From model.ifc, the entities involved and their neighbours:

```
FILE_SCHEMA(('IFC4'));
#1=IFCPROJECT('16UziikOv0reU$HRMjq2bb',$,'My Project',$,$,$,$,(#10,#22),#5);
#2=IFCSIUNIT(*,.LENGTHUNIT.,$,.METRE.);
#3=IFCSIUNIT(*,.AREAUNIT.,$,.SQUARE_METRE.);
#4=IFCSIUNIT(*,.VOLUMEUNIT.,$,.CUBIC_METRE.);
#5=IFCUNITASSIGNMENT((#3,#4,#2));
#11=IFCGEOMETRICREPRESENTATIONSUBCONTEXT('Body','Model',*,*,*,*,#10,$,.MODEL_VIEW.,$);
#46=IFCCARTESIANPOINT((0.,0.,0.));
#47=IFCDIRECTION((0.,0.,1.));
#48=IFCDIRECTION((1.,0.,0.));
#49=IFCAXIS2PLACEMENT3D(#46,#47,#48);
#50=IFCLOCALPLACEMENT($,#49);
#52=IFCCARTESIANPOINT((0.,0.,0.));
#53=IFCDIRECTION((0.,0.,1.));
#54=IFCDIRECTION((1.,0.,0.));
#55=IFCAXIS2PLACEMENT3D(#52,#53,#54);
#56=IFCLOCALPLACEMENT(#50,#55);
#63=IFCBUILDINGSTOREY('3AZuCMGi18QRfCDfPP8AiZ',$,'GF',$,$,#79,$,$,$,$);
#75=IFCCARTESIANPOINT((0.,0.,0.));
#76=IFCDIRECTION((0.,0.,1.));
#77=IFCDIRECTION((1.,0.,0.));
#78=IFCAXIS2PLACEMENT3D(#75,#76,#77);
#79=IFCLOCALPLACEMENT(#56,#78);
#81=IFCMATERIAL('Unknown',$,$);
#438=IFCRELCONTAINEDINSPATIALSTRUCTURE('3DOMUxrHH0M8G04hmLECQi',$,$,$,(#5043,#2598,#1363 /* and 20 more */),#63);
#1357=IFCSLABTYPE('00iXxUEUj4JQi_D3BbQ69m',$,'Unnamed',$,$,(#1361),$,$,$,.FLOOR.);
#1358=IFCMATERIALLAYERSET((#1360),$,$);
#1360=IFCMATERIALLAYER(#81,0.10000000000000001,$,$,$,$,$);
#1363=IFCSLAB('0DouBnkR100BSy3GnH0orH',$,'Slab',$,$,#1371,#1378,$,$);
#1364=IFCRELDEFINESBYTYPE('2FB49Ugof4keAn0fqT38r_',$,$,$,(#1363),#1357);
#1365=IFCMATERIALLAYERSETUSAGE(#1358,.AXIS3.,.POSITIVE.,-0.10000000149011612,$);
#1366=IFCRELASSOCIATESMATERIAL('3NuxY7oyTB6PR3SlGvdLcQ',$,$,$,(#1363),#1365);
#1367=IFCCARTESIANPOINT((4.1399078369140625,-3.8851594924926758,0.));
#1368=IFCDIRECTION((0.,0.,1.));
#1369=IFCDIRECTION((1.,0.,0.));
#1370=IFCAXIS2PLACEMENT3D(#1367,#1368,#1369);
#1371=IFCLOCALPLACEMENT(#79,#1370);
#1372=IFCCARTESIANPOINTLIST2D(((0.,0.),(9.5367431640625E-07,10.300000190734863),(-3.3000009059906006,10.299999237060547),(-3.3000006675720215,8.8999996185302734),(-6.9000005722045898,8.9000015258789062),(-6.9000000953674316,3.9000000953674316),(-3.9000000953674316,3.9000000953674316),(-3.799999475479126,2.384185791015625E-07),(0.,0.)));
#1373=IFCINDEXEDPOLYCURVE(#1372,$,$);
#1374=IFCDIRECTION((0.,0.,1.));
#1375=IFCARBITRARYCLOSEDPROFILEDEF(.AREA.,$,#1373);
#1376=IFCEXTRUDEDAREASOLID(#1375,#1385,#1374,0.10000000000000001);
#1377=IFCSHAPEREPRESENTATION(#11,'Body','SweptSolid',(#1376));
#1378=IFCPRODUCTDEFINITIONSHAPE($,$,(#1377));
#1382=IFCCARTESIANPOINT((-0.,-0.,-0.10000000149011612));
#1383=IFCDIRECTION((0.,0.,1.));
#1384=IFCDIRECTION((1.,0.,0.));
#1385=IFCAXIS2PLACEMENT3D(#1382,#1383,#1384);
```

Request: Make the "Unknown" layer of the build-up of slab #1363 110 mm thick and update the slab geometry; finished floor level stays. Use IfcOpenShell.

```python
import ifcopenshell
import ifcopenshell.util.element
import ifcopenshell.util.representation
import ifcopenshell.util.unit

model = ifcopenshell.open("model.ifc")
unit_scale = ifcopenshell.util.unit.calculate_unit_scale(model)

layer_set = model.by_id(1358)
layer = next(l for l in layer_set.MaterialLayers if l.Material and l.Material.Name == "Unknown")
change = 0.11 / unit_scale - layer.LayerThickness
layer.LayerThickness += change

# Geometry does not follow the layer set by itself.
slabs = [e for e in ifcopenshell.util.element.get_elements_by_material(model, layer_set) if e.is_a("IfcSlab")]
for slab in sorted(slabs, key=lambda e: e.id()):
    body = ifcopenshell.util.representation.get_representation(slab, "Model", "Body")
    solid = body.Items[0]
    old_depth = solid.Depth
    solid.Depth += change
    # Extruded upwards: lower the start of the extrusion so the top stays.
    x, y, z = solid.Position.Location.Coordinates
    solid.Position.Location = model.createIfcCartesianPoint((x, y, z - change))
    print(slab.id(), f"{old_depth:g} -> {solid.Depth:g}")

# The layers are counted up from the underside, which has moved.
for usage in {ifcopenshell.util.element.get_material(slab) for slab in slabs}:
    usage.OffsetFromReferenceLine -= change

model.write("model_rev.ifc")
```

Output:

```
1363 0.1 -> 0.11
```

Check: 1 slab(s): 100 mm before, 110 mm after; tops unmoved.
